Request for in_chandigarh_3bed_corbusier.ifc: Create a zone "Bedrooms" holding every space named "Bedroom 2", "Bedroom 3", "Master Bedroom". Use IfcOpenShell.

First a look at what the model holds.

```python
import ifcopenshell

model = ifcopenshell.open("in_chandigarh_3bed_corbusier.ifc")
print(model.schema)
seen = {}
for space in model.by_type("IfcSpace"):
    seen[space.LongName] = seen.get(space.LongName, 0) + 1
for name, count in sorted(seen.items(), key=str):
    print(count, "x", name)
print("zones:", [z.Name for z in model.by_type("IfcZone")][:20])
```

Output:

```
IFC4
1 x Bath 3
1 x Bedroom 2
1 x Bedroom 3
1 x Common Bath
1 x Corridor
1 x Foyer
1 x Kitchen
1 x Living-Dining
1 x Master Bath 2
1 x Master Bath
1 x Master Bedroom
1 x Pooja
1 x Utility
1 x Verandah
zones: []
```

```python
import ifcopenshell
import ifcopenshell.api.group
import ifcopenshell.api.root

model = ifcopenshell.open("in_chandigarh_3bed_corbusier.ifc")

names = {"Bedroom 2", "Bedroom 3", "Master Bedroom"}
spaces = [s for s in model.by_type("IfcSpace") if s.LongName in names]

zone = ifcopenshell.api.root.create_entity(model, ifc_class="IfcZone", name="Bedrooms")
ifcopenshell.api.group.assign_group(model, products=spaces, group=zone)
print(len(spaces), "spaces in", zone.Name)

model.write("in_chandigarh_3bed_corbusier_rev.ifc")
```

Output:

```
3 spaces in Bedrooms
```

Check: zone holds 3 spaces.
